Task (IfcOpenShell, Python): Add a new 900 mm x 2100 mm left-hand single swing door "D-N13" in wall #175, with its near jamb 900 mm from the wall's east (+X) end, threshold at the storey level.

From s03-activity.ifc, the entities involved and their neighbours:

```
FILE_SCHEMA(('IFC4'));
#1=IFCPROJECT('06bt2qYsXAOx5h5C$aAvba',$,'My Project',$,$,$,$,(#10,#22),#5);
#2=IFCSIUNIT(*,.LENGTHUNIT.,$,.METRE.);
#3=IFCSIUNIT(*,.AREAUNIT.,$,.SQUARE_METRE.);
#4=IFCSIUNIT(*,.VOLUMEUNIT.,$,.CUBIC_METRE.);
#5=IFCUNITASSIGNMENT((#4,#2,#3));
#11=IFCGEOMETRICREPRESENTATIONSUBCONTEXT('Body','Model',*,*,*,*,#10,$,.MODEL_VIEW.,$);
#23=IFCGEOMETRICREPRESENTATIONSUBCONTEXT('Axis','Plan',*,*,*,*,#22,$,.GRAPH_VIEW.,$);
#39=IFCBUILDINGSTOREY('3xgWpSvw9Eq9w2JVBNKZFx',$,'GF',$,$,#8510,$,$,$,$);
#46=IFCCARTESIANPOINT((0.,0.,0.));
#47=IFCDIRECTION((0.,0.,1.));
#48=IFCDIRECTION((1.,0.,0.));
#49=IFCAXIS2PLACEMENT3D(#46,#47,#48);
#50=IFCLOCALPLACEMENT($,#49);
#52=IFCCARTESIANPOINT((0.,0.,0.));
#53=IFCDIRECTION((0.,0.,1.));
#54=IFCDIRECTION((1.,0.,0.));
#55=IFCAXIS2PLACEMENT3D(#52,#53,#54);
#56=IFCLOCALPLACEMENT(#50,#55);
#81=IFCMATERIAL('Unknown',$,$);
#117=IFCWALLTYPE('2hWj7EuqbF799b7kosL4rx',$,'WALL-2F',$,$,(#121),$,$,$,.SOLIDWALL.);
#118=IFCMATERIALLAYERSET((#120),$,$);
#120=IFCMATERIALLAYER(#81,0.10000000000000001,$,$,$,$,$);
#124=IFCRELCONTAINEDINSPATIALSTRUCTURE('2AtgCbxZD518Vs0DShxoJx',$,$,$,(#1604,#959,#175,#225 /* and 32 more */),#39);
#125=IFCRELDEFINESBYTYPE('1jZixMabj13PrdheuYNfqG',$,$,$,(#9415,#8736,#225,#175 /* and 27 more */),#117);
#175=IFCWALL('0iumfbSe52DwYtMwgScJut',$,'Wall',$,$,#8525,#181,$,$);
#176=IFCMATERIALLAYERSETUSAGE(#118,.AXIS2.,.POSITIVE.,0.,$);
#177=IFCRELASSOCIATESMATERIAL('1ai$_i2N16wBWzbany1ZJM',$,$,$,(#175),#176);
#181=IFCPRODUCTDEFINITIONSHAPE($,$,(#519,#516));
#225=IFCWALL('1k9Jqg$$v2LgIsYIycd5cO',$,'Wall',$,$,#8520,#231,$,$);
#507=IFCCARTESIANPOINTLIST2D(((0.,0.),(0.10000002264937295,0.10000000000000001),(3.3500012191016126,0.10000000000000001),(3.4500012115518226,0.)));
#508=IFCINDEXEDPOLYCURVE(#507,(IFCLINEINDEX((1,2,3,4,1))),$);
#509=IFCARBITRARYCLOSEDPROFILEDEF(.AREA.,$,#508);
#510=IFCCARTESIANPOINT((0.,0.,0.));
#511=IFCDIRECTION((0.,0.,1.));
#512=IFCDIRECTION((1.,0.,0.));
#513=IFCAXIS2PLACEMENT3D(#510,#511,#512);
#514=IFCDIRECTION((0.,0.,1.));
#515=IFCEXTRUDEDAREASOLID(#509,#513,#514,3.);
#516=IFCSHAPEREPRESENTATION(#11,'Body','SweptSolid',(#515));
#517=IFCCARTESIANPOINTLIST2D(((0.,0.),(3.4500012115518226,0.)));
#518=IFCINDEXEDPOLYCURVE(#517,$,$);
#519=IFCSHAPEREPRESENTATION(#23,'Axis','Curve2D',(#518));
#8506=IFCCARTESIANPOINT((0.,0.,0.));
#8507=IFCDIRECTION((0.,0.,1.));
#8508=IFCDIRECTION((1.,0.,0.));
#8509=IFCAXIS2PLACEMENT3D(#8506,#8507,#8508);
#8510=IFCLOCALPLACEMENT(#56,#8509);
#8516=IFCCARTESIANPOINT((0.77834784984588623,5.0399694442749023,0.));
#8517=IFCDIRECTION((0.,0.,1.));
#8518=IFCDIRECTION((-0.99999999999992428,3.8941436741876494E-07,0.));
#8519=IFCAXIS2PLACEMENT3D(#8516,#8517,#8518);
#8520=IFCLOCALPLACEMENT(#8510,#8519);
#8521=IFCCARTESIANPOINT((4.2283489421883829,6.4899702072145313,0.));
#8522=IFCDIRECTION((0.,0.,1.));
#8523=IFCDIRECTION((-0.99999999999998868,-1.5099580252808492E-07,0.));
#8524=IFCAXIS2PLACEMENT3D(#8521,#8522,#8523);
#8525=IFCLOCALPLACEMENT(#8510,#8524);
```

```python
import numpy as np
import ifcopenshell
import ifcopenshell.api.feature
import ifcopenshell.api.geometry
import ifcopenshell.api.root
import ifcopenshell.api.spatial
import ifcopenshell.geom
import ifcopenshell.util.element
import ifcopenshell.util.placement
import ifcopenshell.util.representation
import ifcopenshell.util.shape
import ifcopenshell.util.unit

model = ifcopenshell.open("s03-activity.ifc")
unit_scale = ifcopenshell.util.unit.calculate_unit_scale(model)
settings = ifcopenshell.geom.settings()


def volume(element):
    """Net volume in cubic metres, openings subtracted."""
    shape = ifcopenshell.geom.create_shape(settings, element)
    return ifcopenshell.util.shape.get_volume(shape.geometry)


wall = model.by_id(175)
storey = ifcopenshell.util.element.get_container(wall, ifc_class="IfcBuildingStorey")
context = ifcopenshell.util.representation.get_context(model, "Model", "Body", "MODEL_VIEW")
before = volume(wall)

width, height, from_end, sill = 0.9, 2.1, 0.9, 0.0  # metres

# The wall runs along its own X axis, and the end named is its -X end.
wall_shape = ifcopenshell.geom.create_shape(settings, wall)
x, y, z = ifcopenshell.util.shape.get_vertices(wall_shape.geometry).T
start = x.min() + from_end
face, thickness = float(y.min()), float(y.max() - y.min())
wall_matrix = ifcopenshell.util.placement.get_local_placement(wall.ObjectPlacement)
level = ifcopenshell.util.placement.get_local_placement(storey.ObjectPlacement)[2, 3]


def in_wall(x, y):
    """Placement at x, y metres in the wall's axes, at sill height."""
    matrix = wall_matrix.copy()
    matrix[:, 3] = wall_matrix @ np.array([x / unit_scale, y / unit_scale, 0.0, 1.0])
    matrix[2, 3] = level + sill / unit_scale
    return matrix


# Opening: a box that overshoots both wall faces by 50 mm.
opening = ifcopenshell.api.root.create_entity(model, ifc_class="IfcOpeningElement", predefined_type="OPENING")
box = ifcopenshell.api.geometry.add_wall_representation(
    model, context=context, length=width, height=height, thickness=thickness + 0.1
)
ifcopenshell.api.geometry.assign_representation(model, product=opening, representation=box)
ifcopenshell.api.geometry.edit_object_placement(model, product=opening, matrix=in_wall(start, face - 0.05), is_si=False)
ifcopenshell.api.feature.add_feature(model, feature=opening, element=wall)

door = ifcopenshell.api.root.create_entity(model, ifc_class="IfcDoor", name="D-N13", predefined_type="DOOR")
door.OverallWidth, door.OverallHeight = width / unit_scale, height / unit_scale
door.OperationType = "SINGLE_SWING_LEFT"
body = ifcopenshell.api.geometry.add_door_representation(
    model,
    context=context,
    overall_width=door.OverallWidth,
    overall_height=door.OverallHeight,
    operation_type="SINGLE_SWING_LEFT",
    lining_properties={"LiningDepth": thickness / unit_scale, "ThresholdDepth": thickness / unit_scale},
)
ifcopenshell.api.geometry.assign_representation(model, product=door, representation=body)
ifcopenshell.api.spatial.assign_container(model, products=[door], relating_structure=storey)
ifcopenshell.api.feature.add_filling(model, opening=opening, element=door)

# The lining spans the wall, so the door starts at the wall face.
ifcopenshell.api.geometry.edit_object_placement(model, product=door, matrix=in_wall(start, face), is_si=False)

after = volume(wall)

print(f"wall volume {before:.3f} -> {after:.3f} m3")

model.write("s03-activity_rev.ifc")
```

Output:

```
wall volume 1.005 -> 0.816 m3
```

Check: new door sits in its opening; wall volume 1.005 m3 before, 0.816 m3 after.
